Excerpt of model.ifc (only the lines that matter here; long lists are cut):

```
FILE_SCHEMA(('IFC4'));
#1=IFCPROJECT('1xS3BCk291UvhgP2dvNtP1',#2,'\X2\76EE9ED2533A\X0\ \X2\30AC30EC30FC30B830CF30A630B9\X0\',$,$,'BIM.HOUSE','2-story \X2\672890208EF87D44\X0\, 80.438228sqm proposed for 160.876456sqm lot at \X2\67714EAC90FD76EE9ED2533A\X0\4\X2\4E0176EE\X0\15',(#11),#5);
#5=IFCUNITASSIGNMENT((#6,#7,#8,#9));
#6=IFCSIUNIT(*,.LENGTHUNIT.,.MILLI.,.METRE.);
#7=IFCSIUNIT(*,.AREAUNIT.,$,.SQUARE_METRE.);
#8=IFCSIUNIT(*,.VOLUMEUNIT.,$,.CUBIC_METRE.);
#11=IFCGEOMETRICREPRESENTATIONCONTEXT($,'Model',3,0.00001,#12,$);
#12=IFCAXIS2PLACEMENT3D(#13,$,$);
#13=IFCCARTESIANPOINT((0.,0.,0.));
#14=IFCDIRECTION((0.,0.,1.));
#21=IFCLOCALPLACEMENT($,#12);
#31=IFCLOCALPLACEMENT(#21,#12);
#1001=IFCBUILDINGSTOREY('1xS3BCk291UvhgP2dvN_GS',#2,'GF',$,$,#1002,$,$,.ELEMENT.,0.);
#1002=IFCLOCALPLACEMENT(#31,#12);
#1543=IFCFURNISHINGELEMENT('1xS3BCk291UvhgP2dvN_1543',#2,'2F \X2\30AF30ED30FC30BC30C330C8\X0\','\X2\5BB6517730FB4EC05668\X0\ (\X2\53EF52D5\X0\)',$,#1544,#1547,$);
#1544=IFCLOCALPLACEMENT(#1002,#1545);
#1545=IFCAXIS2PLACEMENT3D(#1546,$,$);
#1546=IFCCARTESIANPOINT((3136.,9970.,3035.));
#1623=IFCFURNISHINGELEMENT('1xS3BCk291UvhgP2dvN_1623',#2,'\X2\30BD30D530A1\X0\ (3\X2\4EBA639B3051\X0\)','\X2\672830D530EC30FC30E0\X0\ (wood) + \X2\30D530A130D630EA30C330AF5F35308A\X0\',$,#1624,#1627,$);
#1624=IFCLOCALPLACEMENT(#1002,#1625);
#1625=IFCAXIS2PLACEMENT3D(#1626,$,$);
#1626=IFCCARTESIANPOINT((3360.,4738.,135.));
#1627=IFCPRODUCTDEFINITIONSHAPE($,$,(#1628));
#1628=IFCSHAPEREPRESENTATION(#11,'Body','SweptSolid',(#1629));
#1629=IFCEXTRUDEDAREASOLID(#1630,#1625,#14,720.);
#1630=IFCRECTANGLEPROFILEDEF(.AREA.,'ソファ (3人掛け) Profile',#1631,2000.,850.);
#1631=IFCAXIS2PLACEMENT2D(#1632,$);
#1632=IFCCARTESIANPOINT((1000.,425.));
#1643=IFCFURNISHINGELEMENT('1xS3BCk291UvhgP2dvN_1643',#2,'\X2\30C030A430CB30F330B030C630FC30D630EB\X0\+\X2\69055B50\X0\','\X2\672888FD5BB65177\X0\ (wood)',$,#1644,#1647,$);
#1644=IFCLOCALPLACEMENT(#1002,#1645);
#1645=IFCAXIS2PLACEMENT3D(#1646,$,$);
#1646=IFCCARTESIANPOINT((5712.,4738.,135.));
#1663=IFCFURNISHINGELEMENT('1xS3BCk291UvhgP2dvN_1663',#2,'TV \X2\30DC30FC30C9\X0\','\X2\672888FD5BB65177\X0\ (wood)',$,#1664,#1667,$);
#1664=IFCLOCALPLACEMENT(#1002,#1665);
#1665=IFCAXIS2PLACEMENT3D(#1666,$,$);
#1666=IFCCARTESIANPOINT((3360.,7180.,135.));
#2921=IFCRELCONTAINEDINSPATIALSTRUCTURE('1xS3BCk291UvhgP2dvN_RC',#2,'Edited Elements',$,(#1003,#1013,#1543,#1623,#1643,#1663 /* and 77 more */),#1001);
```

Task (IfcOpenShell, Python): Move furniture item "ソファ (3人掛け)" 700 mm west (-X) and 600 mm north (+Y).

```python
import ifcopenshell
import ifcopenshell.api.geometry
import ifcopenshell.util.placement

model = ifcopenshell.open("model.ifc")

item = model.by_guid("1xS3BCk291UvhgP2dvN_1623")
matrix = ifcopenshell.util.placement.get_local_placement(item.ObjectPlacement)
matrix[0, 3] -= 700.0
matrix[1, 3] += 600.0
ifcopenshell.api.geometry.edit_object_placement(model, product=item, matrix=matrix, is_si=False)

print(ifcopenshell.util.placement.get_local_placement(item.ObjectPlacement).round(3) + 0.0)

model.write("model_edited.ifc")
```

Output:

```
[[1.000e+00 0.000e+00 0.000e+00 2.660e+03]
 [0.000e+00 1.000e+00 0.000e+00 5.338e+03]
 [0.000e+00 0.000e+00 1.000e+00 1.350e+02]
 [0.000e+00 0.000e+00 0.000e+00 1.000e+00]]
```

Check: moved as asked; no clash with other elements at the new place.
